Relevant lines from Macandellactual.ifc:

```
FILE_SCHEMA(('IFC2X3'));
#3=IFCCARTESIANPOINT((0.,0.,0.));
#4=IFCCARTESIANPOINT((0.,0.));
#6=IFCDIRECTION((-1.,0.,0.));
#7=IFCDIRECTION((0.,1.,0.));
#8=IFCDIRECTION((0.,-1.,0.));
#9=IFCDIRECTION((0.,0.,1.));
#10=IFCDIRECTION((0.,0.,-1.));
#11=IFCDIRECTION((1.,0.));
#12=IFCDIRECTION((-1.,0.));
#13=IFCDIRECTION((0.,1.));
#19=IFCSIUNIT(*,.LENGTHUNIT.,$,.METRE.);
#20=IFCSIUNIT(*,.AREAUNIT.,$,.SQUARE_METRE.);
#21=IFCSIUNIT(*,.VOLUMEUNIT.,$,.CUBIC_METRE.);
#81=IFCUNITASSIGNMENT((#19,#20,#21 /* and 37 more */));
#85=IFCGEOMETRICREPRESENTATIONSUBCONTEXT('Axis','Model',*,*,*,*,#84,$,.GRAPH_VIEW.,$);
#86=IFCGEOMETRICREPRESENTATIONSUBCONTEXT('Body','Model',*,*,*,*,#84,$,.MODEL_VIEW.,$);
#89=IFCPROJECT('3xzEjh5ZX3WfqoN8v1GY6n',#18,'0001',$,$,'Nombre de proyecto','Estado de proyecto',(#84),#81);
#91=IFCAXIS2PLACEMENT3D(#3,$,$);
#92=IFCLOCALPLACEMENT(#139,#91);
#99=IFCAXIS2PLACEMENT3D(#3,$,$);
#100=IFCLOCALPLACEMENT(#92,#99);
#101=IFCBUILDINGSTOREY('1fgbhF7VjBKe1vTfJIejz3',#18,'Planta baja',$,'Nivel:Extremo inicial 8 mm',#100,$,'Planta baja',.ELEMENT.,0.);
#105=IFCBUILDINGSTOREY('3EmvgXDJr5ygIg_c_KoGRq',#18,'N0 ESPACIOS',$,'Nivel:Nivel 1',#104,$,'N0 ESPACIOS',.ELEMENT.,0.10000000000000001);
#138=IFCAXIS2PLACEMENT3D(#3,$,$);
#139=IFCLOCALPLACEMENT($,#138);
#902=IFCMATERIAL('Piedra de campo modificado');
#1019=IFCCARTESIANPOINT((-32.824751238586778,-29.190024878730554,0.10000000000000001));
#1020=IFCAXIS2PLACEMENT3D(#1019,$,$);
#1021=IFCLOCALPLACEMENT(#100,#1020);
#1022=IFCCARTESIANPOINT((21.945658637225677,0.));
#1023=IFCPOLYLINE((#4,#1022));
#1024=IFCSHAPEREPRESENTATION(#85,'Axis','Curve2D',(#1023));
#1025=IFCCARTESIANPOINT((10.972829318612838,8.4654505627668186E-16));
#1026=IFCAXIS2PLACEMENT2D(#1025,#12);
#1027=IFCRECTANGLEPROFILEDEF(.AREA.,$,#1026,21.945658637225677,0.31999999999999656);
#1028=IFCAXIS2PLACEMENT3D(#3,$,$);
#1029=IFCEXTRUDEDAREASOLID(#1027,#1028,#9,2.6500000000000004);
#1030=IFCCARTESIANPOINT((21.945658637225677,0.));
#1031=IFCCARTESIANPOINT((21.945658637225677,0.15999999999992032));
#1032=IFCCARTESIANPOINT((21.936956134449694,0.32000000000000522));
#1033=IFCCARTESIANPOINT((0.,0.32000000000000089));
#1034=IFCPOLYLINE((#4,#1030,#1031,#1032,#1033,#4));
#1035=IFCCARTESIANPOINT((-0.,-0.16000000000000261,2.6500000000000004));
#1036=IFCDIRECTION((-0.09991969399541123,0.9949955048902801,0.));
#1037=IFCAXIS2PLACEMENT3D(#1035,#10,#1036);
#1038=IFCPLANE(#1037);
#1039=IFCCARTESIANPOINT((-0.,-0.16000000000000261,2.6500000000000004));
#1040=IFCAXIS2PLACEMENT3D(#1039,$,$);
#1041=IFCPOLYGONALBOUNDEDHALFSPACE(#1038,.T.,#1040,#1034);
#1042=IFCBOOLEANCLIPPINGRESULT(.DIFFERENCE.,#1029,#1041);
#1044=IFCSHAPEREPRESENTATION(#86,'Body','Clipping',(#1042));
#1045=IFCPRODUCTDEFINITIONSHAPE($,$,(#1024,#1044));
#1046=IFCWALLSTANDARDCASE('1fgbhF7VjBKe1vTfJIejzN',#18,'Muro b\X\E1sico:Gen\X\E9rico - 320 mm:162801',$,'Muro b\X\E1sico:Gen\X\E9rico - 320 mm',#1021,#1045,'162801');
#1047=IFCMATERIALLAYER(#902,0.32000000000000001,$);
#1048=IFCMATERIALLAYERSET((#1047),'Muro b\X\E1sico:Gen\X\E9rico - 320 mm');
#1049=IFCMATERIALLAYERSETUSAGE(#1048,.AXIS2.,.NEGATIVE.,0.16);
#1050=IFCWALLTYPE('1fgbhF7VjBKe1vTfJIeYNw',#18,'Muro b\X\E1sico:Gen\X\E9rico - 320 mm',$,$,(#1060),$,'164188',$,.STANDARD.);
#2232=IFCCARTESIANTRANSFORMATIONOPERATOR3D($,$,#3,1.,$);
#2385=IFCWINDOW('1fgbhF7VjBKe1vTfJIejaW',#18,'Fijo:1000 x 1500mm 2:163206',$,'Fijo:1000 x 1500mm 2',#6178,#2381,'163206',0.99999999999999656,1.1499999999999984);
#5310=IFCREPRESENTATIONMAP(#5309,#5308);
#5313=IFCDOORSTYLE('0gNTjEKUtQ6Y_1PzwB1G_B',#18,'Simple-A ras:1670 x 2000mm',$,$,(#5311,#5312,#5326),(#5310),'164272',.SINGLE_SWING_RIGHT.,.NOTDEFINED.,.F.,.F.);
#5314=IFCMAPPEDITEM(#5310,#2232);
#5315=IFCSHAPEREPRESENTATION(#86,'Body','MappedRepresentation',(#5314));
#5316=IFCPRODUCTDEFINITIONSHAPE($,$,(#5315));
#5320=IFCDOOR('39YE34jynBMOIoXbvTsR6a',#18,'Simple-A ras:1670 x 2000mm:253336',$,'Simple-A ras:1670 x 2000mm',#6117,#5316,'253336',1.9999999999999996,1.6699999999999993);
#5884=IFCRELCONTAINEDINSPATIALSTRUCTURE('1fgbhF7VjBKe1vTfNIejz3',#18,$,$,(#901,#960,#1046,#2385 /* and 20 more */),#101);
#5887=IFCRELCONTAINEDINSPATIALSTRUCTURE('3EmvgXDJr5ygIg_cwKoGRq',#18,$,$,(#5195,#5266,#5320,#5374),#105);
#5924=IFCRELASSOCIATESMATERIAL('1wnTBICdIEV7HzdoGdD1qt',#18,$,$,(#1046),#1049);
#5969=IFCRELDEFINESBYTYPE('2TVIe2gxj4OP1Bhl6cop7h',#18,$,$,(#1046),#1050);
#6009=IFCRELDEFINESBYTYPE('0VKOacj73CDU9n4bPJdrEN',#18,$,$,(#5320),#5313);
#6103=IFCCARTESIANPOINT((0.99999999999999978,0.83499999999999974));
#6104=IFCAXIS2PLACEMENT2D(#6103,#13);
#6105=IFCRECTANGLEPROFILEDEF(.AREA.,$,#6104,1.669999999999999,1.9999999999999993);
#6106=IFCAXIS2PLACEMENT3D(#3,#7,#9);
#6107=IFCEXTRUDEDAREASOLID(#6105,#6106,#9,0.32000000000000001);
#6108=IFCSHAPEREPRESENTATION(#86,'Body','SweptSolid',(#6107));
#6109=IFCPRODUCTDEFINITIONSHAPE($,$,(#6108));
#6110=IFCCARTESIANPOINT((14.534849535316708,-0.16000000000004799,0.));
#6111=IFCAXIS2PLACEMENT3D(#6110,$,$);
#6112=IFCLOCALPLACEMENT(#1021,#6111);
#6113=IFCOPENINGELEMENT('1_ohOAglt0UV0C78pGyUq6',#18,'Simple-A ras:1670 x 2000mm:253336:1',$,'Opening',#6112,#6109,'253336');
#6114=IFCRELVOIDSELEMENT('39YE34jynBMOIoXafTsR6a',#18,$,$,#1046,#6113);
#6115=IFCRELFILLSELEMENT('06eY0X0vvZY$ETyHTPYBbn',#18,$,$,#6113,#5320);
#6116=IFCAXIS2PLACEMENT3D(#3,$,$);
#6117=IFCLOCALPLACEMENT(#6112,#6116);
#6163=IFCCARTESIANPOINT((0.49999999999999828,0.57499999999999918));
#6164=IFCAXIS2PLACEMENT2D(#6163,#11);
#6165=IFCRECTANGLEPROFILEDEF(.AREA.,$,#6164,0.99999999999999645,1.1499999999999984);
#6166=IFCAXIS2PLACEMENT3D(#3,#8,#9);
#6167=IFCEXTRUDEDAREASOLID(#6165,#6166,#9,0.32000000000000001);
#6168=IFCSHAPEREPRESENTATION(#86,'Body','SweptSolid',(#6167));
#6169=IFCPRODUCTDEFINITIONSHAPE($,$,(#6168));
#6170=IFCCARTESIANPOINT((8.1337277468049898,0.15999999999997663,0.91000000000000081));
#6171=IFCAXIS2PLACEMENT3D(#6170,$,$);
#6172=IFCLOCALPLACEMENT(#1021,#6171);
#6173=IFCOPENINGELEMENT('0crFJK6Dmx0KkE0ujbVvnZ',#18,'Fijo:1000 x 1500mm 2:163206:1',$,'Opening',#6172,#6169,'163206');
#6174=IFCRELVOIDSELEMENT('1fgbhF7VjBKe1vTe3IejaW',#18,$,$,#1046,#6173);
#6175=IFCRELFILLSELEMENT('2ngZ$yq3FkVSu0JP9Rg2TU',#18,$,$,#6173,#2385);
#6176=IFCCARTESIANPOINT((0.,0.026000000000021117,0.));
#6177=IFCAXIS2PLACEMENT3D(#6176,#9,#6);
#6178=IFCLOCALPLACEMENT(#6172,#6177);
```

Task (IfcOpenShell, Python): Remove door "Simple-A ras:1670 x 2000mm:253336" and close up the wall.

```python
import ifcopenshell
import ifcopenshell.api.feature
import ifcopenshell.api.root
import ifcopenshell.geom
import ifcopenshell.util.shape

model = ifcopenshell.open("Macandellactual.ifc")
settings = ifcopenshell.geom.settings()


def volume(element):
    """Net volume in cubic metres, openings subtracted."""
    shape = ifcopenshell.geom.create_shape(settings, element)
    return ifcopenshell.util.shape.get_volume(shape.geometry)


door = model.by_guid("39YE34jynBMOIoXbvTsR6a")
opening = door.FillsVoids[0].RelatingOpeningElement
wall = opening.VoidsElements[0].RelatingBuildingElement
before = volume(wall)

ifcopenshell.api.root.remove_product(model, product=door)
ifcopenshell.api.feature.remove_feature(model, feature=opening)

after = volume(wall)

print(f"wall volume {before:.3f} -> {after:.3f} m3")

model.write("Macandellactual_v2.ifc")
```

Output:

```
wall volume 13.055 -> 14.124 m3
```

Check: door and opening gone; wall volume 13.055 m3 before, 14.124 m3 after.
